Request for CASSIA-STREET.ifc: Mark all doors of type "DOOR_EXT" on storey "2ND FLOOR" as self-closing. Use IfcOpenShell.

First a look at what the model holds.

```python
import ifcopenshell
import ifcopenshell.util.element

model = ifcopenshell.open("CASSIA-STREET.ifc")
print(model.schema)
storey = next(s for s in model.by_type("IfcBuildingStorey") if s.Name == "2ND FLOOR")
doors = [e for e in ifcopenshell.util.element.get_decomposition(storey) if e.is_a("IfcDoor")]
seen = {}
for e in doors:
    element_type = ifcopenshell.util.element.get_type(e)
    key = (element_type.Name if element_type != e and element_type else None, ifcopenshell.util.element.get_pset(e, "Pset_DoorCommon", "SelfClosing"))
    seen[key] = seen.get(key, 0) + 1
for (name, value), count in sorted(seen.items(), key=str):
    print(count, "x", name, "|", value)
```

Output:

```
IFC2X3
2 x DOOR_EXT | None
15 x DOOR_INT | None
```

```python
import ifcopenshell
import ifcopenshell.api.pset
import ifcopenshell.util.element

model = ifcopenshell.open("CASSIA-STREET.ifc")

storey = next(s for s in model.by_type("IfcBuildingStorey") if s.Name == "2ND FLOOR")
doors = [e for e in ifcopenshell.util.element.get_decomposition(storey) if e.is_a("IfcDoor")]

count = 0
for e in doors:
    element_type = ifcopenshell.util.element.get_type(e)
    if element_type in (None, e) or element_type.Name != "DOOR_EXT":
        continue
    # add_pset returns the element's existing set when there is one.
    pset = ifcopenshell.api.pset.add_pset(model, product=e, name="Pset_DoorCommon")
    ifcopenshell.api.pset.edit_pset(model, pset=pset, properties={"SelfClosing": True})
    count += 1

print(count, "doors updated")

model.write("CASSIA-STREET-out.ifc")
```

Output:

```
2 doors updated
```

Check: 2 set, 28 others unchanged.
